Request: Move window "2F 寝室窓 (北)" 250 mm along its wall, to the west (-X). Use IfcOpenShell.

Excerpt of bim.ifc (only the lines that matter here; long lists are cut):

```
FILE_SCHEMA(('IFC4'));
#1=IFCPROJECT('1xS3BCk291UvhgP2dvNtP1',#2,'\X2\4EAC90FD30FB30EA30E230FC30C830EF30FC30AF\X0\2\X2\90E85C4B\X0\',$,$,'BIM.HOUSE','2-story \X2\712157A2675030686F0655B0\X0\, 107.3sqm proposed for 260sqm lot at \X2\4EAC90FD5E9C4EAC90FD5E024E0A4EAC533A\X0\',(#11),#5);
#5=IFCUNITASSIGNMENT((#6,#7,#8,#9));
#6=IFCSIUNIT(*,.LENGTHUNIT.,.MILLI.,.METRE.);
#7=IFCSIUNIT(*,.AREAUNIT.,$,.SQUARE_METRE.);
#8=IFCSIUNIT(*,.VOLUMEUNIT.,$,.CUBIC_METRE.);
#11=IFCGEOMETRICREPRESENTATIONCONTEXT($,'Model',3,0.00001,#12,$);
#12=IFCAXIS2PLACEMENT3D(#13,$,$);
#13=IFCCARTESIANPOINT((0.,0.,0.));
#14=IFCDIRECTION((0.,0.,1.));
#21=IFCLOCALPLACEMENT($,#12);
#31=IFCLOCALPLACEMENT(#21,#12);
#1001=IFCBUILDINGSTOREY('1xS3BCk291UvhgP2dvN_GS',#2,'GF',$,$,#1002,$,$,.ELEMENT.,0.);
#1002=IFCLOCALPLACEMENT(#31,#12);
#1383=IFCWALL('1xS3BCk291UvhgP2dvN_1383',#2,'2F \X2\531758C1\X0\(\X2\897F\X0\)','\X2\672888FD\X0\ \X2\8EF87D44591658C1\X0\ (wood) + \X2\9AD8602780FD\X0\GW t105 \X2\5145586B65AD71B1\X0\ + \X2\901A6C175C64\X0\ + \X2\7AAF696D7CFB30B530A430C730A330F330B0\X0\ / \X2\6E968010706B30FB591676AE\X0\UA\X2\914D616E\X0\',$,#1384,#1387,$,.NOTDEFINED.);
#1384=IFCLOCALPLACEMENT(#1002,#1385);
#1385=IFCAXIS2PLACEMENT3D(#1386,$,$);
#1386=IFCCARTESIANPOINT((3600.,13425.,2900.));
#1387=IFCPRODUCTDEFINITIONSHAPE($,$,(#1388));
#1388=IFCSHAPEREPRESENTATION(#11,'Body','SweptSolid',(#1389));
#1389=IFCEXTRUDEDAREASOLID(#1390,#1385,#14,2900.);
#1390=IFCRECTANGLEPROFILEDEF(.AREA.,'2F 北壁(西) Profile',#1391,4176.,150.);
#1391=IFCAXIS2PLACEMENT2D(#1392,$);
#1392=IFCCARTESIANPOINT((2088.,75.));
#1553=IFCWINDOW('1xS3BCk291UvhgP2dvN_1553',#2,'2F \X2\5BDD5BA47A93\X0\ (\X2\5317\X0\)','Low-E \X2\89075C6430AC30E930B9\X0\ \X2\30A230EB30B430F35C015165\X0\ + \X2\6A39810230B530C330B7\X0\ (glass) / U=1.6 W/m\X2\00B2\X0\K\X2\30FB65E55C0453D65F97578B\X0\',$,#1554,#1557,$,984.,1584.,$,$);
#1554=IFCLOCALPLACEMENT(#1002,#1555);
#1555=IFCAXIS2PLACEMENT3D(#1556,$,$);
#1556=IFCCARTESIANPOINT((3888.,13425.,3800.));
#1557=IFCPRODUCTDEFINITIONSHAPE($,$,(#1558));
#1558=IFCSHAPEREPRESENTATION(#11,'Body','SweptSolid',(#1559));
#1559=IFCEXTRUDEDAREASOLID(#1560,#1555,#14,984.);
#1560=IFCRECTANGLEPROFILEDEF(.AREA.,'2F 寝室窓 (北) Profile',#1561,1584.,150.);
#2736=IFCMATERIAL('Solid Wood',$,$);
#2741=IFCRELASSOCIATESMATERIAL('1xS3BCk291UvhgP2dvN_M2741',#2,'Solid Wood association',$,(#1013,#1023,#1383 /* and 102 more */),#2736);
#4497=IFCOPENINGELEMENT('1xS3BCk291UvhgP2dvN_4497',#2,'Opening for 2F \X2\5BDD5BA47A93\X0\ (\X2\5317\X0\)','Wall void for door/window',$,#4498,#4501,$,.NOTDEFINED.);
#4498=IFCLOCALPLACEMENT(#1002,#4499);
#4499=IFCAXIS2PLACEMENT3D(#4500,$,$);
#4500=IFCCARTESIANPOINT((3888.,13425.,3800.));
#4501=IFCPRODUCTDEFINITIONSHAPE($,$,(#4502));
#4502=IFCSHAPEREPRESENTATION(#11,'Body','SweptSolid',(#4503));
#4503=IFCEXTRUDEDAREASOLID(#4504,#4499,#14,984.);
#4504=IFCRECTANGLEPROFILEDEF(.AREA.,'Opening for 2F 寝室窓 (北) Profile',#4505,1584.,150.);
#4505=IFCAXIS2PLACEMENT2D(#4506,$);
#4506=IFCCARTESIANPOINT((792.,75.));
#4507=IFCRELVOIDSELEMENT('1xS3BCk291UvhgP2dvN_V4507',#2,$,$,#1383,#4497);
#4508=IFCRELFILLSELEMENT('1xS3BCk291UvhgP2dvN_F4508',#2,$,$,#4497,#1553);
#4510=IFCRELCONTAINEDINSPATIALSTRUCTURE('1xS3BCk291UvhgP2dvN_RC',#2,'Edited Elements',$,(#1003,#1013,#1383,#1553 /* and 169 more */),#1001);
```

```python
import ifcopenshell
import ifcopenshell.api.geometry
import ifcopenshell.util.placement
import ifcopenshell.util.unit

model = ifcopenshell.open("bim.ifc")
unit_scale = ifcopenshell.util.unit.calculate_unit_scale(model)

window = model.by_id(1553)
opening = window.FillsVoids[0].RelatingOpeningElement
wall = opening.VoidsElements[0].RelatingBuildingElement

wall_matrix = ifcopenshell.util.placement.get_local_placement(wall.ObjectPlacement)
shift = wall_matrix[:3, 0] * -0.25 / unit_scale
before = ifcopenshell.util.placement.get_local_placement(window.ObjectPlacement)[:3, 3].copy()

# The window is not placed relative to its opening, so move both.
for product in (opening, window):
    matrix = ifcopenshell.util.placement.get_local_placement(product.ObjectPlacement)
    matrix[:3, 3] += shift
    ifcopenshell.api.geometry.edit_object_placement(model, product=product, matrix=matrix, is_si=False)

after = ifcopenshell.util.placement.get_local_placement(window.ObjectPlacement)[:3, 3]
print("window moved by", (after - before).round(3) + 0.0)

model.write("bim_edited.ifc")
```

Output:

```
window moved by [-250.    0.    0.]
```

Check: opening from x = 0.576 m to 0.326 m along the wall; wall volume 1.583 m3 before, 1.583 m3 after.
